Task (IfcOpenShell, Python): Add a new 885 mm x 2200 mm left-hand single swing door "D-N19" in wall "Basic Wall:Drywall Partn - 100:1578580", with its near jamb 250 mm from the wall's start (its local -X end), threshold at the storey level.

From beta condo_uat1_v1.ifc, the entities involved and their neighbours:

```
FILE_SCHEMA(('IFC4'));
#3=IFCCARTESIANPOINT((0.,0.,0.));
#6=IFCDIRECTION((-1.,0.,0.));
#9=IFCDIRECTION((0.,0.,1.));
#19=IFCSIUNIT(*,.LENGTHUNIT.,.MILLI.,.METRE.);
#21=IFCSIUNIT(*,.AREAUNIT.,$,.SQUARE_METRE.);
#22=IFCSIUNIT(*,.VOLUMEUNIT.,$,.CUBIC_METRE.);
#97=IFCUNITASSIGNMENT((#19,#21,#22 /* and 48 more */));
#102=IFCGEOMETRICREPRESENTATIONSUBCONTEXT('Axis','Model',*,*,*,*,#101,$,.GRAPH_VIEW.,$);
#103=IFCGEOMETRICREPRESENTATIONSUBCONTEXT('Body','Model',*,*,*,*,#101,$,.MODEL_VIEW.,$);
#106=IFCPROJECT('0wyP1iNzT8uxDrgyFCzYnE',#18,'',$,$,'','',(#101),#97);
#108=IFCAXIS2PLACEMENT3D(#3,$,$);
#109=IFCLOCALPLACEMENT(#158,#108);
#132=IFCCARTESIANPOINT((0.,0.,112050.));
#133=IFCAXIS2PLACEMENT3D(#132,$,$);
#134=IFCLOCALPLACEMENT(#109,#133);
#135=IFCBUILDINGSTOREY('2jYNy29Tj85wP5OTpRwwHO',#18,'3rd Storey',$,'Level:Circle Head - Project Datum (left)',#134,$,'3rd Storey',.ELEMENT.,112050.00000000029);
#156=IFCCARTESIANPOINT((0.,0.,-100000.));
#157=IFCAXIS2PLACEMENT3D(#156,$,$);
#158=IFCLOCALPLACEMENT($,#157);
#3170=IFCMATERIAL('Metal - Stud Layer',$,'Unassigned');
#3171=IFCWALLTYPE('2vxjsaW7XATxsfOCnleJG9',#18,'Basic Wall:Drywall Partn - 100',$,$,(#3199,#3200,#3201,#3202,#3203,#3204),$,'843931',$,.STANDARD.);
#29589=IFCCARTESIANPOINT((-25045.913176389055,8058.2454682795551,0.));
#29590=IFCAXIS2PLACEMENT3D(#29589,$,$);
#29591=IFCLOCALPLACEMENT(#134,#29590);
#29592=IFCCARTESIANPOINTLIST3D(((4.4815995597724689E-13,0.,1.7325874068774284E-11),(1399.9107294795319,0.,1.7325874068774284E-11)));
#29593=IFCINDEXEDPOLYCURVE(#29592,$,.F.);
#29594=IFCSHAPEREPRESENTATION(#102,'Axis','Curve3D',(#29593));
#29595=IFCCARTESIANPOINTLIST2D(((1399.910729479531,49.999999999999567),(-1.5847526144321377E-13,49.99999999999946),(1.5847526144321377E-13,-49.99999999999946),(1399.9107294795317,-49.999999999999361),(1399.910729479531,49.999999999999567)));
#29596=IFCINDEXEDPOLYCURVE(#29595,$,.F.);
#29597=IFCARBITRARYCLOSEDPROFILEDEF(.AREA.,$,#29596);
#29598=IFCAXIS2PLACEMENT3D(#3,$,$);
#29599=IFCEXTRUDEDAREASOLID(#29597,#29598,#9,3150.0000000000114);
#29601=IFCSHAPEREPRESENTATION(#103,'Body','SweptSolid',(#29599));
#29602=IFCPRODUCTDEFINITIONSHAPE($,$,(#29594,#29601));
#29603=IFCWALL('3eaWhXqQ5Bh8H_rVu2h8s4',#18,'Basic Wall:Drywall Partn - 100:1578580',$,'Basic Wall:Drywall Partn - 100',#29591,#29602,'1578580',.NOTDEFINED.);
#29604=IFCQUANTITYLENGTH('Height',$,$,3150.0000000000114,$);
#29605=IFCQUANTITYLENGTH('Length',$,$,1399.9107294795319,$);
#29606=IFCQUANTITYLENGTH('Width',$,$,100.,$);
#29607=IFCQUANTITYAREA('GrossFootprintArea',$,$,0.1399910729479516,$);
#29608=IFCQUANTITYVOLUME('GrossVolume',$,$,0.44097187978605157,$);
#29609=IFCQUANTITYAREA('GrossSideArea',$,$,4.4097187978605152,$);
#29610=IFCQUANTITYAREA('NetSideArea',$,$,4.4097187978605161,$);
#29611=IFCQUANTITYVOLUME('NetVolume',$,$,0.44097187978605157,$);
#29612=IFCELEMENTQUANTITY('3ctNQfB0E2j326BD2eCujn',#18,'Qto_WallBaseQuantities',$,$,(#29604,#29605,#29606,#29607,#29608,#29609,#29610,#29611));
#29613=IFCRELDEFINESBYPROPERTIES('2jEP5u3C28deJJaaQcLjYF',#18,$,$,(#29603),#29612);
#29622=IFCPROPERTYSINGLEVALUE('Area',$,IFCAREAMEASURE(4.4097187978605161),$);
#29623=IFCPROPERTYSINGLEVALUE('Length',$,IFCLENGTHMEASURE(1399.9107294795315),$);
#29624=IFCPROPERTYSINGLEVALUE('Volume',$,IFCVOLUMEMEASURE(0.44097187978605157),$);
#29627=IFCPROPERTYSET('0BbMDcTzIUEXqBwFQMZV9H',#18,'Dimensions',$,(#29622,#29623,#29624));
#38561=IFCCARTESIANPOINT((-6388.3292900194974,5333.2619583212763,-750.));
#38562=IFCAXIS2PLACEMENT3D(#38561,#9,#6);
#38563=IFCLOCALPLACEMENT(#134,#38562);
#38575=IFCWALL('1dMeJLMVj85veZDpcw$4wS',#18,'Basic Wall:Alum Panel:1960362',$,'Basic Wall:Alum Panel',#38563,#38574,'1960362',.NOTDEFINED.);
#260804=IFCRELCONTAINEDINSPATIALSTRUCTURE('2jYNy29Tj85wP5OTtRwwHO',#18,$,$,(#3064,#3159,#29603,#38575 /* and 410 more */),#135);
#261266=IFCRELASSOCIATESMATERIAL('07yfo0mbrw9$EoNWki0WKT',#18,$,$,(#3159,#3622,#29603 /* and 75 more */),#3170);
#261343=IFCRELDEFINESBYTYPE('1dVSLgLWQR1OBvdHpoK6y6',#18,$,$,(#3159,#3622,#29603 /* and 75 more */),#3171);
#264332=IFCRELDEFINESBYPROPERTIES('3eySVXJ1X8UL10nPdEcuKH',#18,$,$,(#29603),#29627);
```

```python
import numpy as np
import ifcopenshell
import ifcopenshell.api.feature
import ifcopenshell.api.geometry
import ifcopenshell.api.pset
import ifcopenshell.api.root
import ifcopenshell.api.spatial
import ifcopenshell.geom
import ifcopenshell.util.element
import ifcopenshell.util.placement
import ifcopenshell.util.representation
import ifcopenshell.util.shape
import ifcopenshell.util.unit

model = ifcopenshell.open("beta condo_uat1_v1.ifc")
unit_scale = ifcopenshell.util.unit.calculate_unit_scale(model)
area_scale = ifcopenshell.util.unit.calculate_unit_scale(model, "AREAUNIT")
volume_scale = ifcopenshell.util.unit.calculate_unit_scale(model, "VOLUMEUNIT")
settings = ifcopenshell.geom.settings()


def volume(element):
    """Net volume in cubic metres, openings subtracted."""
    shape = ifcopenshell.geom.create_shape(settings, element)
    return ifcopenshell.util.shape.get_volume(shape.geometry)


wall = model.by_guid("3eaWhXqQ5Bh8H_rVu2h8s4")
storey = ifcopenshell.util.element.get_container(wall, ifc_class="IfcBuildingStorey")
context = ifcopenshell.util.representation.get_context(model, "Model", "Body", "MODEL_VIEW")
before = volume(wall)

width, height, from_end, sill = 0.885, 2.2, 0.25, 0.0  # metres

# The wall runs along its own X axis, and the end named is its -X end.
wall_shape = ifcopenshell.geom.create_shape(settings, wall)
x, y, z = ifcopenshell.util.shape.get_vertices(wall_shape.geometry).T
start = x.min() + from_end
face, thickness = float(y.min()), float(y.max() - y.min())
wall_matrix = ifcopenshell.util.placement.get_local_placement(wall.ObjectPlacement)
level = ifcopenshell.util.placement.get_local_placement(storey.ObjectPlacement)[2, 3]


def in_wall(x, y):
    """Placement at x, y metres in the wall's axes, at sill height."""
    matrix = wall_matrix.copy()
    matrix[:, 3] = wall_matrix @ np.array([x / unit_scale, y / unit_scale, 0.0, 1.0])
    matrix[2, 3] = level + sill / unit_scale
    return matrix


# Opening: a box that overshoots both wall faces by 50 mm.
opening = ifcopenshell.api.root.create_entity(model, ifc_class="IfcOpeningElement", predefined_type="OPENING")
box = ifcopenshell.api.geometry.add_wall_representation(
    model, context=context, length=width, height=height, thickness=thickness + 0.1
)
ifcopenshell.api.geometry.assign_representation(model, product=opening, representation=box)
ifcopenshell.api.geometry.edit_object_placement(model, product=opening, matrix=in_wall(start, face - 0.05), is_si=False)
ifcopenshell.api.feature.add_feature(model, feature=opening, element=wall)

door = ifcopenshell.api.root.create_entity(model, ifc_class="IfcDoor", name="D-N19", predefined_type="DOOR")
door.OverallWidth, door.OverallHeight = width / unit_scale, height / unit_scale
door.OperationType = "SINGLE_SWING_LEFT"
body = ifcopenshell.api.geometry.add_door_representation(
    model,
    context=context,
    overall_width=door.OverallWidth,
    overall_height=door.OverallHeight,
    operation_type="SINGLE_SWING_LEFT",
    lining_properties={"LiningDepth": thickness / unit_scale, "ThresholdDepth": thickness / unit_scale},
)
ifcopenshell.api.geometry.assign_representation(model, product=door, representation=body)
ifcopenshell.api.spatial.assign_container(model, products=[door], relating_structure=storey)
ifcopenshell.api.feature.add_filling(model, opening=opening, element=door)

# The lining spans the wall, so the door starts at the wall face.
ifcopenshell.api.geometry.edit_object_placement(model, product=door, matrix=in_wall(start, face), is_si=False)

after = volume(wall)

# Update the wall's stored quantities.
qto = model.by_id(ifcopenshell.util.element.get_pset(wall, "Qto_WallBaseQuantities", should_inherit=False)["id"])
ifcopenshell.api.pset.edit_qto(model, qto=qto, properties={
    "NetSideArea": after / thickness / area_scale,
    "NetVolume": after / volume_scale,
})
pset = model.by_id(ifcopenshell.util.element.get_pset(wall, "Dimensions", should_inherit=False)["id"])
ifcopenshell.api.pset.edit_pset(model, pset=pset, properties={
    "Area": model.create_entity("IfcAreaMeasure", after / thickness / area_scale),
    "Volume": model.create_entity("IfcVolumeMeasure", after / volume_scale),
})

print(f"wall volume {before:.3f} -> {after:.3f} m3")

model.write("beta condo_uat1_v1_updated.ifc")
```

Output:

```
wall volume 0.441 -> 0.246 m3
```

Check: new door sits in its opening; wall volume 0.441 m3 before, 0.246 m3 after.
